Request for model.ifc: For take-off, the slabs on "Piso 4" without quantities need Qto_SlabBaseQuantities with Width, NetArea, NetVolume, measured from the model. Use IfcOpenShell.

First a look at what the model holds.

```python
import ifcopenshell
import ifcopenshell.util.element
import ifcopenshell.util.unit

model = ifcopenshell.open("model.ifc")
print(model.schema)
for unit_type in ("LENGTHUNIT", "AREAUNIT", "VOLUMEUNIT"):
    print(unit_type, ifcopenshell.util.unit.calculate_unit_scale(model, unit_type))
storey = next(s for s in model.by_type("IfcBuildingStorey") if s.Name == "Piso 4")
slabs = [e for e in ifcopenshell.util.element.get_decomposition(storey) if e.is_a("IfcSlab")]
for e in sorted(slabs, key=lambda e: e.id()):
    print(e.id(), e.is_a(), e.Name, list(ifcopenshell.util.element.get_psets(e, qtos_only=True)), sep=" | ")
```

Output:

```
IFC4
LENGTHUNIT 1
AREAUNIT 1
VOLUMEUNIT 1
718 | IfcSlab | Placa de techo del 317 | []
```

```python
import ifcopenshell
import ifcopenshell.api.pset
import ifcopenshell.geom
import ifcopenshell.util.element
import ifcopenshell.util.shape
import ifcopenshell.util.unit

model = ifcopenshell.open("model.ifc")
unit_scale = ifcopenshell.util.unit.calculate_unit_scale(model)
area_scale = ifcopenshell.util.unit.calculate_unit_scale(model, "AREAUNIT")
volume_scale = ifcopenshell.util.unit.calculate_unit_scale(model, "VOLUMEUNIT")
settings = ifcopenshell.geom.settings()

storey = next(s for s in model.by_type("IfcBuildingStorey") if s.Name == "Piso 4")
slabs = [e for e in ifcopenshell.util.element.get_decomposition(storey) if e.is_a("IfcSlab")]

for e in sorted(slabs, key=lambda e: e.id()):
    if ifcopenshell.util.element.get_psets(e, qtos_only=True, should_inherit=False):
        continue
    # Geometry comes back in metres, in the element's own axes.
    shape = ifcopenshell.geom.create_shape(settings, e)
    values = {
        "Width": ifcopenshell.util.shape.get_z(shape.geometry) / unit_scale,
        "NetArea": ifcopenshell.util.shape.get_footprint_area(shape.geometry) / area_scale,
        "NetVolume": ifcopenshell.util.shape.get_volume(shape.geometry) / volume_scale,
    }
    qto = ifcopenshell.api.pset.add_qto(model, product=e, name="Qto_SlabBaseQuantities")
    ifcopenshell.api.pset.edit_qto(model, qto=qto, properties=values)
    print(e.id(), {k: round(v, 3) for k, v in values.items()})

model.write("model_updated.ifc")
```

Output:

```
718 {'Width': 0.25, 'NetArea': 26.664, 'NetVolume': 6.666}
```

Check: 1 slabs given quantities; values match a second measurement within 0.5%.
